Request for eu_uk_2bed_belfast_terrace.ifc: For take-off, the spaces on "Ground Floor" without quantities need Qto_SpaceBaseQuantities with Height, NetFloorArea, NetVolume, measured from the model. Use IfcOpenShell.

First a look at what the model holds.

```python
import ifcopenshell
import ifcopenshell.util.element
import ifcopenshell.util.unit

model = ifcopenshell.open("eu_uk_2bed_belfast_terrace.ifc")
print(model.schema)
for unit_type in ("LENGTHUNIT", "AREAUNIT", "VOLUMEUNIT"):
    print(unit_type, ifcopenshell.util.unit.calculate_unit_scale(model, unit_type))
storey = next(s for s in model.by_type("IfcBuildingStorey") if s.Name == "Ground Floor")
spaces = [e for e in ifcopenshell.util.element.get_decomposition(storey) if e.is_a("IfcSpace")]
for e in sorted(spaces, key=lambda e: e.id()):
    print(e.id(), e.is_a(), e.Name, list(ifcopenshell.util.element.get_psets(e, qtos_only=True)), sep=" | ")
```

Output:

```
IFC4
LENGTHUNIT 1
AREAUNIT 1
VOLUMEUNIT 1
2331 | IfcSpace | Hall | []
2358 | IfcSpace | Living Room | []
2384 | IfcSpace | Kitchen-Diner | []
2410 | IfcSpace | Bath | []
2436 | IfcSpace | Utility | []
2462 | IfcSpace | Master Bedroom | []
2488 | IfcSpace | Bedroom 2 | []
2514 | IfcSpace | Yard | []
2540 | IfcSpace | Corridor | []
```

```python
import ifcopenshell
import ifcopenshell.api.pset
import ifcopenshell.geom
import ifcopenshell.util.element
import ifcopenshell.util.shape
import ifcopenshell.util.unit

model = ifcopenshell.open("eu_uk_2bed_belfast_terrace.ifc")
unit_scale = ifcopenshell.util.unit.calculate_unit_scale(model)
area_scale = ifcopenshell.util.unit.calculate_unit_scale(model, "AREAUNIT")
volume_scale = ifcopenshell.util.unit.calculate_unit_scale(model, "VOLUMEUNIT")
settings = ifcopenshell.geom.settings()

storey = next(s for s in model.by_type("IfcBuildingStorey") if s.Name == "Ground Floor")
spaces = [e for e in ifcopenshell.util.element.get_decomposition(storey) if e.is_a("IfcSpace")]

for e in sorted(spaces, key=lambda e: e.id()):
    if ifcopenshell.util.element.get_psets(e, qtos_only=True, should_inherit=False):
        continue
    # Geometry comes back in metres, in the element's own axes.
    shape = ifcopenshell.geom.create_shape(settings, e)
    values = {
        "Height": ifcopenshell.util.shape.get_z(shape.geometry) / unit_scale,
        "NetFloorArea": ifcopenshell.util.shape.get_footprint_area(shape.geometry) / area_scale,
        "NetVolume": ifcopenshell.util.shape.get_volume(shape.geometry) / volume_scale,
    }
    qto = ifcopenshell.api.pset.add_qto(model, product=e, name="Qto_SpaceBaseQuantities")
    ifcopenshell.api.pset.edit_qto(model, qto=qto, properties=values)
    print(e.id(), {k: round(v, 3) for k, v in values.items()})

model.write("eu_uk_2bed_belfast_terrace_updated.ifc")
```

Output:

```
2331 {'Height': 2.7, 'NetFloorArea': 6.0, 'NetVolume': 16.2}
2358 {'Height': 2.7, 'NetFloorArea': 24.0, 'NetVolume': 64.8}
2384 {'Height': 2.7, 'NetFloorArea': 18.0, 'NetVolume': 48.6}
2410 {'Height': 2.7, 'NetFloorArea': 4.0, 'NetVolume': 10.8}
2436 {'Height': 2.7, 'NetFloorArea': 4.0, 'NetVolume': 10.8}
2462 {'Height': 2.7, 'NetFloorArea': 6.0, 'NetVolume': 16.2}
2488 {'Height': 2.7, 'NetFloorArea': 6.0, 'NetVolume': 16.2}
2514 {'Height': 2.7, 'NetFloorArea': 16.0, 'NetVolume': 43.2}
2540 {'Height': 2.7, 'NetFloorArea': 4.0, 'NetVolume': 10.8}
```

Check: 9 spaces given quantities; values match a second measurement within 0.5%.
